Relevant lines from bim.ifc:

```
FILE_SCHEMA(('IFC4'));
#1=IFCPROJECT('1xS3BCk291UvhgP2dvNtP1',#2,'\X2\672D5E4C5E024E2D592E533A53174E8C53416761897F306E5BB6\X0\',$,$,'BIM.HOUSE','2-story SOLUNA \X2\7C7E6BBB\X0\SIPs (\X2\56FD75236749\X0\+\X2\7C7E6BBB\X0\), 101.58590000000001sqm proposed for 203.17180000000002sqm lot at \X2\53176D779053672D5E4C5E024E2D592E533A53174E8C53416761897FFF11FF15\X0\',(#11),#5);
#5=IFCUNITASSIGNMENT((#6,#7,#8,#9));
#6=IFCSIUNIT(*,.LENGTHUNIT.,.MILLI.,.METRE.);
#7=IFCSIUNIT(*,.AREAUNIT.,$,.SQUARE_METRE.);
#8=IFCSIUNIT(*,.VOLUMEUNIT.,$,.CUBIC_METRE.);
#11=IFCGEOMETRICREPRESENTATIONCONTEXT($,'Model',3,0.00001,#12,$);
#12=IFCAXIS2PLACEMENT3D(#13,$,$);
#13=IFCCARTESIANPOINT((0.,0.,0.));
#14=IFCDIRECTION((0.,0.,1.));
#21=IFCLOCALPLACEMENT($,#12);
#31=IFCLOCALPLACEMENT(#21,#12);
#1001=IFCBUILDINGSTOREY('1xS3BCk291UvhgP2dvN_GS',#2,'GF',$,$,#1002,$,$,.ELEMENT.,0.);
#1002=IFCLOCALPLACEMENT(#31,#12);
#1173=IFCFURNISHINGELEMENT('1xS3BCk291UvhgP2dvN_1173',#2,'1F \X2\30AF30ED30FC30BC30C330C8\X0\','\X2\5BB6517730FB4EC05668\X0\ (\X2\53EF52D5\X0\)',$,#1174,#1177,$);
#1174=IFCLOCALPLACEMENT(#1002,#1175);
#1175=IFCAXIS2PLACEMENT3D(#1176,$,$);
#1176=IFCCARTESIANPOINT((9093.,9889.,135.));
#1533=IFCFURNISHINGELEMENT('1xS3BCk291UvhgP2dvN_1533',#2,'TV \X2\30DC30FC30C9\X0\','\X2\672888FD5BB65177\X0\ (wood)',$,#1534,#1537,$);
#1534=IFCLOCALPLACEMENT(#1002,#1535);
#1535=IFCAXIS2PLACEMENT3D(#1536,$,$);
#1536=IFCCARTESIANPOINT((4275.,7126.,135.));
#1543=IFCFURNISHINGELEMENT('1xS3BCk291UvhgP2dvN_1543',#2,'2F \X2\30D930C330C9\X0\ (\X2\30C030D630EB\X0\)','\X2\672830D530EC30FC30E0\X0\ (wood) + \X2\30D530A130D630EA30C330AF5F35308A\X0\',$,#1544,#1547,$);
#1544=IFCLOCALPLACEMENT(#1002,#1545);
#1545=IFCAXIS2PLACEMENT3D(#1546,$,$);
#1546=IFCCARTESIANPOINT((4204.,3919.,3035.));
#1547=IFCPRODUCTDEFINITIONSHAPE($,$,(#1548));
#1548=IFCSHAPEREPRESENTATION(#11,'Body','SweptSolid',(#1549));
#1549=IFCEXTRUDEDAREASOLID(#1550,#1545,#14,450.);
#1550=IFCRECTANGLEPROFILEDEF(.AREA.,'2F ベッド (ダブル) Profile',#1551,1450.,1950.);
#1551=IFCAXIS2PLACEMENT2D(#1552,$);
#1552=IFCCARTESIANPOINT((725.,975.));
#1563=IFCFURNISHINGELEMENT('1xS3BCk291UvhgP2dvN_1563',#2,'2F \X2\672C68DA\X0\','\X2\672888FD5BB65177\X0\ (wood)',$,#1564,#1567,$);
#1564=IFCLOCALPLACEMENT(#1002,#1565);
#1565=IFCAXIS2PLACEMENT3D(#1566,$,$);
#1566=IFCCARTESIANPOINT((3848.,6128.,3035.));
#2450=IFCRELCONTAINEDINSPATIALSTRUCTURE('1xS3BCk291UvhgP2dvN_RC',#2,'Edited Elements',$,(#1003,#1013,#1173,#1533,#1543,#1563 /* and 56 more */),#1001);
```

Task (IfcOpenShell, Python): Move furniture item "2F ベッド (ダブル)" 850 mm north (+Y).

```python
import ifcopenshell
import ifcopenshell.api.geometry
import ifcopenshell.util.placement

model = ifcopenshell.open("bim.ifc")

item = model.by_guid("1xS3BCk291UvhgP2dvN_1543")
matrix = ifcopenshell.util.placement.get_local_placement(item.ObjectPlacement)
matrix[1, 3] += 850.0
ifcopenshell.api.geometry.edit_object_placement(model, product=item, matrix=matrix, is_si=False)

print(ifcopenshell.util.placement.get_local_placement(item.ObjectPlacement).round(3) + 0.0)

model.write("bim_edited.ifc")
```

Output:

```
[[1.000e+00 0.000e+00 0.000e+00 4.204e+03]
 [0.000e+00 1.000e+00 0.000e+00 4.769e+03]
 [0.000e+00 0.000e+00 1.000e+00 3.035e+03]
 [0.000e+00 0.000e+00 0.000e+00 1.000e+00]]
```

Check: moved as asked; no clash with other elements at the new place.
